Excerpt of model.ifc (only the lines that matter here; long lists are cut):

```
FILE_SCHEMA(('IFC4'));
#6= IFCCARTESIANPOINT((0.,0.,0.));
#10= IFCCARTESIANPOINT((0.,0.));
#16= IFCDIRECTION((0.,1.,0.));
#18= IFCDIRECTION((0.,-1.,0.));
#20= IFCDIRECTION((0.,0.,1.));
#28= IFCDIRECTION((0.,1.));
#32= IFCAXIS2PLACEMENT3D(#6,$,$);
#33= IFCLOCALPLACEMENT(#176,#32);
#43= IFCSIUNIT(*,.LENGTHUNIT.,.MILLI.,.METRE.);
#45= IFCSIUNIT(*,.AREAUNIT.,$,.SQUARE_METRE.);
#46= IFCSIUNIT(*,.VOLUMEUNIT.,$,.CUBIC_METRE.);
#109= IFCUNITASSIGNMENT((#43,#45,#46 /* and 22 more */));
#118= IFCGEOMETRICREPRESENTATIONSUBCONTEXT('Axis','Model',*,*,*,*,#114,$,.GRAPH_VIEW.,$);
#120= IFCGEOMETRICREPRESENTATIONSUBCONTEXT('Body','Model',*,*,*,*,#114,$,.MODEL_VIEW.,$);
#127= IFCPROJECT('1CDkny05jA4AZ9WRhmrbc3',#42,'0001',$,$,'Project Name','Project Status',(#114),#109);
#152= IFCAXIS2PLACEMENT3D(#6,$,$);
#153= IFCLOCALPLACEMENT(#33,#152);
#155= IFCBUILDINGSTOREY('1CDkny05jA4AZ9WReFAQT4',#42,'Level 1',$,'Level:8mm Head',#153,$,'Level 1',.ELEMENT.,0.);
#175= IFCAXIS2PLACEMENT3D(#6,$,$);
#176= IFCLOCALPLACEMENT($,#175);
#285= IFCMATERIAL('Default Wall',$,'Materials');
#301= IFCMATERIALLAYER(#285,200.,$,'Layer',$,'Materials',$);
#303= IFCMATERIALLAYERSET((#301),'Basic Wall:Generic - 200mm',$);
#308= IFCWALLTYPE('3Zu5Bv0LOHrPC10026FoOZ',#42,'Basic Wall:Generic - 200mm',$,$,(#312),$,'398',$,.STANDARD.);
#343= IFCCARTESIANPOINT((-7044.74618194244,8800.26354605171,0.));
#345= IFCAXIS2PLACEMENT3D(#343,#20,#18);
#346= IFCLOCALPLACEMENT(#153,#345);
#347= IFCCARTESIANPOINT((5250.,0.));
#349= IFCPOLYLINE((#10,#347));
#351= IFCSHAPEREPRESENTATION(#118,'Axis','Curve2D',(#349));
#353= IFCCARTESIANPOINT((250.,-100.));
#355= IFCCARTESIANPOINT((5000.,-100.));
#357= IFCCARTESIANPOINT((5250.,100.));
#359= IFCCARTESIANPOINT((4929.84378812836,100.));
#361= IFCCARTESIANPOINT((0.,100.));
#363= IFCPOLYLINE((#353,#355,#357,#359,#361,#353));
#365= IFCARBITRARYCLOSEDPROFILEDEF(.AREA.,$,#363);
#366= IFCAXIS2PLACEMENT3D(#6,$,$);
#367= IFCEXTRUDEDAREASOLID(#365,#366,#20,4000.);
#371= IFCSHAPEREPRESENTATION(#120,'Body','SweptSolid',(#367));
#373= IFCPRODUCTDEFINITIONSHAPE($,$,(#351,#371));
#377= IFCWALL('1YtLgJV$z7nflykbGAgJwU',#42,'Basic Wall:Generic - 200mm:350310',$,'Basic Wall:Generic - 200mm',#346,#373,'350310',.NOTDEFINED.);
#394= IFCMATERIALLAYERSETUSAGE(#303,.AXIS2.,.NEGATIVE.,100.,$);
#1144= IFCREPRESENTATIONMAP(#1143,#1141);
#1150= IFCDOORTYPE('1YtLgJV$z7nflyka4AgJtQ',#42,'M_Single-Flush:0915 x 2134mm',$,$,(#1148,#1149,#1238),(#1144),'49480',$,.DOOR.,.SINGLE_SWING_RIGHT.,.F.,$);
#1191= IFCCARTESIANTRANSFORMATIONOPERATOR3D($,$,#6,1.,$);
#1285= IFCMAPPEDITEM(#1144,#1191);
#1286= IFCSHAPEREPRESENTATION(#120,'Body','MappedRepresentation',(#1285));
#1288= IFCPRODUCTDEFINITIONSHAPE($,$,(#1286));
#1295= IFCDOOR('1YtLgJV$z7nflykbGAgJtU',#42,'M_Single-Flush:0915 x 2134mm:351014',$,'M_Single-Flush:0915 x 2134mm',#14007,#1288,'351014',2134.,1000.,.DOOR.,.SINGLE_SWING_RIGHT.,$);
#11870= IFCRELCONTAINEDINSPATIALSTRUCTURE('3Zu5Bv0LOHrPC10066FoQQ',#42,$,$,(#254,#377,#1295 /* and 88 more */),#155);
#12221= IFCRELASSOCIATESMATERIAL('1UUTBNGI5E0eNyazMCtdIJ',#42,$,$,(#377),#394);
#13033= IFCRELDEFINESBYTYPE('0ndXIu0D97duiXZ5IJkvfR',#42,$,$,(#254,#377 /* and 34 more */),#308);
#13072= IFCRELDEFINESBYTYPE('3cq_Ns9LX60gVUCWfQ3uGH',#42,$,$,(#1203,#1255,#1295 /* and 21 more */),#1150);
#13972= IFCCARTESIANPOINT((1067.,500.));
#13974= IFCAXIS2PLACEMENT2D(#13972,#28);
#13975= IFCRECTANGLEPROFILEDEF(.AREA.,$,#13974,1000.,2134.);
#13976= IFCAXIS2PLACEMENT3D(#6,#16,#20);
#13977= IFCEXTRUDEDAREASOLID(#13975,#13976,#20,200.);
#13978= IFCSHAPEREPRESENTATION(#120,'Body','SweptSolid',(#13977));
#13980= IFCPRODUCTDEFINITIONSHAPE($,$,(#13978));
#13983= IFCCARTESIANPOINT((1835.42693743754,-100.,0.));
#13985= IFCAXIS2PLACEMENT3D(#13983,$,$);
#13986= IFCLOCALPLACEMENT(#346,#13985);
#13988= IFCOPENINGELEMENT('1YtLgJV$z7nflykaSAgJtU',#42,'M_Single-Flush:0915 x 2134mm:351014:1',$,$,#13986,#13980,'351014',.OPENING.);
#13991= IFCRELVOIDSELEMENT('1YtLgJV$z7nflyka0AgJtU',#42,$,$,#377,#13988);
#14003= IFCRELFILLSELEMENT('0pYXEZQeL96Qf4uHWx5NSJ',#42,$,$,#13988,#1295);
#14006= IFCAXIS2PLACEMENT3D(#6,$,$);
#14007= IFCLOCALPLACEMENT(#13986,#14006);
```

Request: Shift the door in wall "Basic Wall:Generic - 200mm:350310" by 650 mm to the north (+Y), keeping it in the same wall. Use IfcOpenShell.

```python
import ifcopenshell
import ifcopenshell.api.geometry
import ifcopenshell.util.placement
import ifcopenshell.util.unit

model = ifcopenshell.open("model.ifc")
unit_scale = ifcopenshell.util.unit.calculate_unit_scale(model)

door = model.by_guid("1YtLgJV$z7nflykbGAgJtU")
opening = door.FillsVoids[0].RelatingOpeningElement
wall = opening.VoidsElements[0].RelatingBuildingElement

wall_matrix = ifcopenshell.util.placement.get_local_placement(wall.ObjectPlacement)
shift = wall_matrix[:3, 0] * -0.65 / unit_scale
before = ifcopenshell.util.placement.get_local_placement(door.ObjectPlacement)[:3, 3].copy()

# The door is placed relative to its opening, so it follows when the opening moves.
matrix = ifcopenshell.util.placement.get_local_placement(opening.ObjectPlacement)
matrix[:3, 3] += shift
ifcopenshell.api.geometry.edit_object_placement(
    model, product=opening, matrix=matrix, is_si=False, should_transform_children=True
)

after = ifcopenshell.util.placement.get_local_placement(door.ObjectPlacement)[:3, 3]
print("door moved by", (after - before).round(3) + 0.0)

model.write("model_v2.ifc")
```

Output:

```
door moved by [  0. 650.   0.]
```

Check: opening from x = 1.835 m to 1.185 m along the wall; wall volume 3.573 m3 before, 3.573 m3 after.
